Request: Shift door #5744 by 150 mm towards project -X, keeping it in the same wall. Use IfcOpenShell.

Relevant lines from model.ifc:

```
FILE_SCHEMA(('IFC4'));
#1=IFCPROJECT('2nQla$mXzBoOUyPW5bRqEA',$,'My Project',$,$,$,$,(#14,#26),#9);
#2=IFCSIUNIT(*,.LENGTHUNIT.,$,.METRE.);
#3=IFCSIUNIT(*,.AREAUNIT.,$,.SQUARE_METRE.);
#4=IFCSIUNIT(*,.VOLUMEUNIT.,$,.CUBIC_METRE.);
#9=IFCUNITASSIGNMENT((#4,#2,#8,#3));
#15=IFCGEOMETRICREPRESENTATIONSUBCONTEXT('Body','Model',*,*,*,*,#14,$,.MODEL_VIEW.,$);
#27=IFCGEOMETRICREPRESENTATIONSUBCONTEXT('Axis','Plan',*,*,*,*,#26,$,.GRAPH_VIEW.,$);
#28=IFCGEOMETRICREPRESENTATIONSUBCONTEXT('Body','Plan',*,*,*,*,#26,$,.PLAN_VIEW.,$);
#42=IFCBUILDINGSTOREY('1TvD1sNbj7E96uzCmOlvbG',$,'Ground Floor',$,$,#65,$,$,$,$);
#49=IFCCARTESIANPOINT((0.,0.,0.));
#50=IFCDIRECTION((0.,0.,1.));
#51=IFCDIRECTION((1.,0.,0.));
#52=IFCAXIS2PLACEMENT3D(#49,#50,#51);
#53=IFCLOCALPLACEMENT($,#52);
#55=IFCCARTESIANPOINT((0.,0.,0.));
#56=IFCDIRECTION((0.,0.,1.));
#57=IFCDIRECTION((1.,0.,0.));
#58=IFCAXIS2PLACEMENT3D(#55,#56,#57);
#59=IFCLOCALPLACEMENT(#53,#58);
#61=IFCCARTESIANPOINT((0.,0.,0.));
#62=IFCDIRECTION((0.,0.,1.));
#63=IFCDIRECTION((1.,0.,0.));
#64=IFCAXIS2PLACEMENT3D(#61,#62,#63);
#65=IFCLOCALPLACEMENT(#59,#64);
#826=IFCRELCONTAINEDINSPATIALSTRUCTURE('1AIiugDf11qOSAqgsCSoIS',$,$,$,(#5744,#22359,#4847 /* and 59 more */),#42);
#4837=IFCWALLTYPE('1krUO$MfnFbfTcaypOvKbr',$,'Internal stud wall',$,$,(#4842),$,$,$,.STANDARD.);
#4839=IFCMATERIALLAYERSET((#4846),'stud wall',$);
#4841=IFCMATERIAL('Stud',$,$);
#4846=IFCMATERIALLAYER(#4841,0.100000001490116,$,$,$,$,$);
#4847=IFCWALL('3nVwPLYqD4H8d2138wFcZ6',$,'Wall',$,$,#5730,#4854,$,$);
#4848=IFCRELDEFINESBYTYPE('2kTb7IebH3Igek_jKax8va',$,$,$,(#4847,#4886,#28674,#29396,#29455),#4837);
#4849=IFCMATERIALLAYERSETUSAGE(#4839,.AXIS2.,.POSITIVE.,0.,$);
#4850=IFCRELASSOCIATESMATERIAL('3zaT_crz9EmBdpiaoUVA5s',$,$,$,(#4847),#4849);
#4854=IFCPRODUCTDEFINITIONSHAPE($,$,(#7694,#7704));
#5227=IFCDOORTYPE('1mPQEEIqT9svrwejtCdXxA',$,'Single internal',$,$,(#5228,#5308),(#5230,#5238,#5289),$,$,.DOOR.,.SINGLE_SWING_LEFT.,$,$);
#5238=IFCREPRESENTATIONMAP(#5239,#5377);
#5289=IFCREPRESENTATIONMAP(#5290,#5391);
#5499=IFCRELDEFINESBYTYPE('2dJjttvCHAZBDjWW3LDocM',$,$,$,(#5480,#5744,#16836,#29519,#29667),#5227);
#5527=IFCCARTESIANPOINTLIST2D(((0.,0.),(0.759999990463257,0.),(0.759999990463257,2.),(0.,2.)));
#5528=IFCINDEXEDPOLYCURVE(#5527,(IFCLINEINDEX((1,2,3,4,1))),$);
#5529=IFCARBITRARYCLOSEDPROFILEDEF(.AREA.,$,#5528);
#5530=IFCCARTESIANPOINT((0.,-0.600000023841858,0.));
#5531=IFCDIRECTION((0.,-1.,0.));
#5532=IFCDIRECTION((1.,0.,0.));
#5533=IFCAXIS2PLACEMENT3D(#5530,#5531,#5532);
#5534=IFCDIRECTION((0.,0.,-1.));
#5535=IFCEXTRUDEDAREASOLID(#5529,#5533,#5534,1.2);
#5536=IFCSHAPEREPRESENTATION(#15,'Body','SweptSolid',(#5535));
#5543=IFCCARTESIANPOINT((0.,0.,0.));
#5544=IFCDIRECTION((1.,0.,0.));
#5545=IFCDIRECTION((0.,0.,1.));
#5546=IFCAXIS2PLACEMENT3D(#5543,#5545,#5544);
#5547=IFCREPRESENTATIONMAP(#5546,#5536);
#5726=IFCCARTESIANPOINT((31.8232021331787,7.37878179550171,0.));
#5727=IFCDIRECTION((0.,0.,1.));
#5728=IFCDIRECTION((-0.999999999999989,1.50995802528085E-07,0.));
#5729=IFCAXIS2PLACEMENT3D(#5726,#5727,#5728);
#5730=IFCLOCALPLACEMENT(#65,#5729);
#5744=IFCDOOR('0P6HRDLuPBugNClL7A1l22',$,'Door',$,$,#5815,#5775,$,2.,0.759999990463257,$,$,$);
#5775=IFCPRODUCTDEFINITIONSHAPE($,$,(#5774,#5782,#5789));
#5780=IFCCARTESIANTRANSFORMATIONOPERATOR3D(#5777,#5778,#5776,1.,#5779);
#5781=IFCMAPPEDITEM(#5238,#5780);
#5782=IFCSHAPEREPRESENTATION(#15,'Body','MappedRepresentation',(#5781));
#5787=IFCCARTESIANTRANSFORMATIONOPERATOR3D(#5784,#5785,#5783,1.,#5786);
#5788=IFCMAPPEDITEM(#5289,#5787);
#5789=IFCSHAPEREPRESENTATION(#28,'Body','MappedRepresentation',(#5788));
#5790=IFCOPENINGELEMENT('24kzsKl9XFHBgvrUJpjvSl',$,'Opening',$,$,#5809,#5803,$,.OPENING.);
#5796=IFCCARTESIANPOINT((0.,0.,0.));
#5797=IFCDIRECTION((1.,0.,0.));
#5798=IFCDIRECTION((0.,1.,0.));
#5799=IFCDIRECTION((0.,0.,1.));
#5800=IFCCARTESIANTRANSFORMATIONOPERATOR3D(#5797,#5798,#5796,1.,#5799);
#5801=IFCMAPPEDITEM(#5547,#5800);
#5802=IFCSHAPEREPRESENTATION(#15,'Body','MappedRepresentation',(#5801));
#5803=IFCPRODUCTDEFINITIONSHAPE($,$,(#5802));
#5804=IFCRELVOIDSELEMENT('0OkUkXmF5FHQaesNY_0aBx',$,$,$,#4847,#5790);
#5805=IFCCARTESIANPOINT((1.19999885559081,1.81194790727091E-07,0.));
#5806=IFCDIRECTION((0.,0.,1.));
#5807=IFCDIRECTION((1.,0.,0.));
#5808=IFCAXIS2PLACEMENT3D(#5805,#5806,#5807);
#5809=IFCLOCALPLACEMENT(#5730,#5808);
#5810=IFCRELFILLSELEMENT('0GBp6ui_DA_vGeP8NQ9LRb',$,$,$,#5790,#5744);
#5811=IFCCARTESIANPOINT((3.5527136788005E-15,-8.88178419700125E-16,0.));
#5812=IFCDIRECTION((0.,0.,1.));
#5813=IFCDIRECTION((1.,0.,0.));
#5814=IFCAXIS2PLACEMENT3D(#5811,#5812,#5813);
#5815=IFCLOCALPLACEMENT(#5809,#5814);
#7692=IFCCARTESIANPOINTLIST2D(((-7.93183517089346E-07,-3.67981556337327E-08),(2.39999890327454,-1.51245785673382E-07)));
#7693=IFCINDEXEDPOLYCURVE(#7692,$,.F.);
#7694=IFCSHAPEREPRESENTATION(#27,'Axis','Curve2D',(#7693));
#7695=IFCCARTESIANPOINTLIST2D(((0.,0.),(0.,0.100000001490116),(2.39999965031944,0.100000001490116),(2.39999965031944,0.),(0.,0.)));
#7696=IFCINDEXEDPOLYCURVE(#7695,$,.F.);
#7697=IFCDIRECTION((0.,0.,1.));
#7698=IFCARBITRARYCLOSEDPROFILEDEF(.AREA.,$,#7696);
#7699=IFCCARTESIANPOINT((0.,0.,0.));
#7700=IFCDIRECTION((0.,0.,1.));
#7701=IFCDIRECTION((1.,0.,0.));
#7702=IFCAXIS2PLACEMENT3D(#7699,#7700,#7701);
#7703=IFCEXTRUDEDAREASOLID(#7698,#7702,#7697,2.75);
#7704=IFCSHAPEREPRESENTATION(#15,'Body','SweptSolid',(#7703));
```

```python
import ifcopenshell
import ifcopenshell.api.geometry
import ifcopenshell.util.placement
import ifcopenshell.util.unit

model = ifcopenshell.open("model.ifc")
unit_scale = ifcopenshell.util.unit.calculate_unit_scale(model)

door = model.by_guid("0P6HRDLuPBugNClL7A1l22")
opening = door.FillsVoids[0].RelatingOpeningElement
wall = opening.VoidsElements[0].RelatingBuildingElement

wall_matrix = ifcopenshell.util.placement.get_local_placement(wall.ObjectPlacement)
shift = wall_matrix[:3, 0] * 0.15 / unit_scale
before = ifcopenshell.util.placement.get_local_placement(door.ObjectPlacement)[:3, 3].copy()

# The door is placed relative to its opening, so it follows when the opening moves.
matrix = ifcopenshell.util.placement.get_local_placement(opening.ObjectPlacement)
matrix[:3, 3] += shift
ifcopenshell.api.geometry.edit_object_placement(
    model, product=opening, matrix=matrix, is_si=False, should_transform_children=True
)

after = ifcopenshell.util.placement.get_local_placement(door.ObjectPlacement)[:3, 3]
print("door moved by", (after - before).round(3) + 0.0)

model.write("model_updated.ifc")
```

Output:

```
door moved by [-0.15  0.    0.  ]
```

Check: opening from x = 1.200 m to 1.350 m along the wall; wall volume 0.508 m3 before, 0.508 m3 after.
